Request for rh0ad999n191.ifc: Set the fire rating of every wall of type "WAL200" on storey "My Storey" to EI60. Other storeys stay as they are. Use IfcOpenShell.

First a look at what the model holds.

```python
import ifcopenshell
import ifcopenshell.util.element

model = ifcopenshell.open("rh0ad999n191.ifc")
print(model.schema)
storey = next(s for s in model.by_type("IfcBuildingStorey") if s.Name == "My Storey")
walls = [e for e in ifcopenshell.util.element.get_decomposition(storey) if e.is_a("IfcWall")]
seen = {}
for e in walls:
    element_type = ifcopenshell.util.element.get_type(e)
    key = (element_type.Name if element_type != e and element_type else None, ifcopenshell.util.element.get_pset(e, "Pset_WallCommon", "FireRating"))
    seen[key] = seen.get(key, 0) + 1
for (name, value), count in sorted(seen.items(), key=str):
    print(count, "x", name, "|", value)
```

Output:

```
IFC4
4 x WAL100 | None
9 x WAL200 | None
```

```python
import ifcopenshell
import ifcopenshell.api.pset
import ifcopenshell.util.element

model = ifcopenshell.open("rh0ad999n191.ifc")

storey = next(s for s in model.by_type("IfcBuildingStorey") if s.Name == "My Storey")
walls = [e for e in ifcopenshell.util.element.get_decomposition(storey) if e.is_a("IfcWall")]

count = 0
for e in walls:
    element_type = ifcopenshell.util.element.get_type(e)
    if element_type in (None, e) or element_type.Name != "WAL200":
        continue
    # add_pset returns the element's existing set when there is one.
    pset = ifcopenshell.api.pset.add_pset(model, product=e, name="Pset_WallCommon")
    ifcopenshell.api.pset.edit_pset(model, pset=pset, properties={"FireRating": "EI60"})
    count += 1

print(count, "walls updated")

model.write("rh0ad999n191_updated.ifc")
```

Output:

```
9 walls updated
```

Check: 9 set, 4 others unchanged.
